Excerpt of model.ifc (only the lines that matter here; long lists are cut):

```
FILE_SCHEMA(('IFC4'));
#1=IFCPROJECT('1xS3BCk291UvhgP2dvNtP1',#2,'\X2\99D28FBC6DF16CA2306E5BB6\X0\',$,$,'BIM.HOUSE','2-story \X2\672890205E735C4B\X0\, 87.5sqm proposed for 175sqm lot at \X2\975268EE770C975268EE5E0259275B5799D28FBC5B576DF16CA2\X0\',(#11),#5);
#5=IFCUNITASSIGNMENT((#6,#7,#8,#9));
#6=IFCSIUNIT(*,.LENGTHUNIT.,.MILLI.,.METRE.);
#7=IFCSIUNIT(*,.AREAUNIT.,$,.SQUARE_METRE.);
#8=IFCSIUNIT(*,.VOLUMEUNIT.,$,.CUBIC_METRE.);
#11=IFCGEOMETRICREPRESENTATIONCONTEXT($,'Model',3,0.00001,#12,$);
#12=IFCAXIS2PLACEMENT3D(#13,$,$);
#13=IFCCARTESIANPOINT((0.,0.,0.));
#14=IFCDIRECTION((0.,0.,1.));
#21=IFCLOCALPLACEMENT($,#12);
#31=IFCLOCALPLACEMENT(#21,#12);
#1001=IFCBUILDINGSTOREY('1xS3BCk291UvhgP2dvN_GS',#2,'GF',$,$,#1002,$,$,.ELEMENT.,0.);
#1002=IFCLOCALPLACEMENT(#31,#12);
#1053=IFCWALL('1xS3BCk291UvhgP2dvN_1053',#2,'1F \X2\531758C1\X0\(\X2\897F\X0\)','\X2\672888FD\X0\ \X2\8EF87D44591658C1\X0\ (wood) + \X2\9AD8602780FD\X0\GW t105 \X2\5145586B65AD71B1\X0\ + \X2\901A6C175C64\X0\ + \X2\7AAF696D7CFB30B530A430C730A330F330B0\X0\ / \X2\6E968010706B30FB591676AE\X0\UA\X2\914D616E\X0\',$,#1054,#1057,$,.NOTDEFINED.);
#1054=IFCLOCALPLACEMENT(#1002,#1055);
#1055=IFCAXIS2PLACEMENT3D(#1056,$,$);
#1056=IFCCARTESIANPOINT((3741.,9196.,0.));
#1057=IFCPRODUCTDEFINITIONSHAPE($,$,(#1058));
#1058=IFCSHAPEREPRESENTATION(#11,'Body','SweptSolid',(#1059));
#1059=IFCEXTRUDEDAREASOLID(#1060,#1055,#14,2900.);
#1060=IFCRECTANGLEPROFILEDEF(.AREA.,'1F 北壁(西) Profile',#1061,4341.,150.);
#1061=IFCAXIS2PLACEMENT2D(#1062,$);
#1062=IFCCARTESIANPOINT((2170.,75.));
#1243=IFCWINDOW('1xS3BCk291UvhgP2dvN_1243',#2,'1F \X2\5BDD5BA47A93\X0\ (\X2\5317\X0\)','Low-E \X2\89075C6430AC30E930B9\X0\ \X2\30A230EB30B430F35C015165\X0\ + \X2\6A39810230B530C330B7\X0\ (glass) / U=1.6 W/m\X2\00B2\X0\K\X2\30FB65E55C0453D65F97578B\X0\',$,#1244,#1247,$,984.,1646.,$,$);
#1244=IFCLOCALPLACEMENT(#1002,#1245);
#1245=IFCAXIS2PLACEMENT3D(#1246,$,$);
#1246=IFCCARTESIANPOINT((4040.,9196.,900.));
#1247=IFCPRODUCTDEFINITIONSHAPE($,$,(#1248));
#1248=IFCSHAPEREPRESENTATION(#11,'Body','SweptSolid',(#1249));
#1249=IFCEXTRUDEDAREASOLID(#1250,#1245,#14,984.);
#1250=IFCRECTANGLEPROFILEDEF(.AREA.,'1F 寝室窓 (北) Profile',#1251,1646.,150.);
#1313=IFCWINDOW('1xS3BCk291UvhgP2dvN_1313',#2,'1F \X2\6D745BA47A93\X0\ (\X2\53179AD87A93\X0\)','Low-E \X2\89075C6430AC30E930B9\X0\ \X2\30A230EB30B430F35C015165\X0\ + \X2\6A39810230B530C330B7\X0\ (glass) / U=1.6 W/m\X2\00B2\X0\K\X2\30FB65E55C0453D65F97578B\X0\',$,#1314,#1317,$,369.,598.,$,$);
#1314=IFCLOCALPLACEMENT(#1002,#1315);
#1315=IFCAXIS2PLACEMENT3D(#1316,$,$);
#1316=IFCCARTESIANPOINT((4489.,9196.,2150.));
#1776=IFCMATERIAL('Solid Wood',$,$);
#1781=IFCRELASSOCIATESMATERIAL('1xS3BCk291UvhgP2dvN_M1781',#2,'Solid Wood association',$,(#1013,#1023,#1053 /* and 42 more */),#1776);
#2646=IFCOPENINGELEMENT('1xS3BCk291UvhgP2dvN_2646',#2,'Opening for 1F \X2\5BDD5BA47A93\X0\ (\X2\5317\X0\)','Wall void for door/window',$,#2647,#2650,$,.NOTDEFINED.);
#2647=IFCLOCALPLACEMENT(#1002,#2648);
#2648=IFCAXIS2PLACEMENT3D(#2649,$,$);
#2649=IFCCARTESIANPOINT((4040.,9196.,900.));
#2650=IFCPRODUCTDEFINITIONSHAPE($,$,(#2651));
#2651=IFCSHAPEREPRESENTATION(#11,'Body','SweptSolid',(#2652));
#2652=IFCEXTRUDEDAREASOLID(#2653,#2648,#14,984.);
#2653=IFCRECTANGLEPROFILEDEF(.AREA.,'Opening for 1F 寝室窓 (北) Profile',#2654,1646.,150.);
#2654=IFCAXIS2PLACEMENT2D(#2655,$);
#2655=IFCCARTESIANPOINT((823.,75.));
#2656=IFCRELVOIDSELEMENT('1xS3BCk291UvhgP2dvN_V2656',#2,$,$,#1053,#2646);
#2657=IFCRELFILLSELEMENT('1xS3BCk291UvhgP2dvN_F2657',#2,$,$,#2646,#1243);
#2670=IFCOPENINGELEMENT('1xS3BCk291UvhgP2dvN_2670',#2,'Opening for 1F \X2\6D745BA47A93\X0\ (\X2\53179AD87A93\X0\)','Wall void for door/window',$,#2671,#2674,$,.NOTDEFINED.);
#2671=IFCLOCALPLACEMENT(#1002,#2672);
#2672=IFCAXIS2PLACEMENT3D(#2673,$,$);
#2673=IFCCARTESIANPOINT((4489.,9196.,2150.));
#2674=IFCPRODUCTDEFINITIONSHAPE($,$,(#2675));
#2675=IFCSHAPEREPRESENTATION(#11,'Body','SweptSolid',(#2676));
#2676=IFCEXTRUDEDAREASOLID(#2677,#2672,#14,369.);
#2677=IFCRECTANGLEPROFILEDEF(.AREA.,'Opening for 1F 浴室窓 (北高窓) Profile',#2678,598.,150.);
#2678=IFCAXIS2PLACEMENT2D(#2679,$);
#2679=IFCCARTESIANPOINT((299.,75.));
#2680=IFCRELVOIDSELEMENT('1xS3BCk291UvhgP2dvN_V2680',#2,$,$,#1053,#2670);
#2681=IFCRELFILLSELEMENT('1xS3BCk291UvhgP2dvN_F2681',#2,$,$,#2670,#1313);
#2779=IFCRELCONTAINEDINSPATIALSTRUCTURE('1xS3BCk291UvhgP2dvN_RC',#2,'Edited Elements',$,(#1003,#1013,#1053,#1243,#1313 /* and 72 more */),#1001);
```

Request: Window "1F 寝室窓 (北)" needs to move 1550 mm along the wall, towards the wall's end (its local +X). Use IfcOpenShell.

```python
import ifcopenshell
import ifcopenshell.api.geometry
import ifcopenshell.util.placement

model = ifcopenshell.open("model.ifc")

window = model.by_id(1243)
opening = window.FillsVoids[0].RelatingOpeningElement
wall = opening.VoidsElements[0].RelatingBuildingElement

wall_matrix = ifcopenshell.util.placement.get_local_placement(wall.ObjectPlacement)
shift = wall_matrix[:3, 0] * 1550.0
before = ifcopenshell.util.placement.get_local_placement(window.ObjectPlacement)[:3, 3].copy()

# The window is not placed relative to its opening, so move both.
for product in (opening, window):
    matrix = ifcopenshell.util.placement.get_local_placement(product.ObjectPlacement)
    matrix[:3, 3] += shift
    ifcopenshell.api.geometry.edit_object_placement(model, product=product, matrix=matrix, is_si=False)

after = ifcopenshell.util.placement.get_local_placement(window.ObjectPlacement)[:3, 3]
print("window moved by", (after - before).round(3) + 0.0)

model.write("model_updated.ifc")
```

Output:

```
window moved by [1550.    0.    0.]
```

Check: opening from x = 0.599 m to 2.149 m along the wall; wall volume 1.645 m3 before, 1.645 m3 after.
